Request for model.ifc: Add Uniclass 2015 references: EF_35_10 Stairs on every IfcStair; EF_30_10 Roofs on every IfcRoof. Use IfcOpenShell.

First a look at what the model holds.

```python
import ifcopenshell

model = ifcopenshell.open("model.ifc")
print(model.schema)
print("classifications:", [c.Name for c in model.by_type("IfcClassification")])
for ifc_class in ("IfcDoor", "IfcRoof", "IfcStair", "IfcWall", "IfcWindow"):
    print(ifc_class, len(model.by_type(ifc_class)))
```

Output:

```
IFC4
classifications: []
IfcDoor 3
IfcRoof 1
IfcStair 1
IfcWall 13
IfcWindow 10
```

```python
import ifcopenshell
import ifcopenshell.api.classification

model = ifcopenshell.open("model.ifc")

system = ifcopenshell.api.classification.add_classification(model, classification="Uniclass 2015")

codes = {
    "IfcStair": ("EF_35_10", "Stairs"),
    "IfcRoof": ("EF_30_10", "Roofs"),
}
for ifc_class, (code, name) in codes.items():
    products = model.by_type(ifc_class)
    ifcopenshell.api.classification.add_reference(
        model, products=products, classification=system, identification=code, name=name
    )
    print(code, len(products))

model.write("model_v2.ifc")
```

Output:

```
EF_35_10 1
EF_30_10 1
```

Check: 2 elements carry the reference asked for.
